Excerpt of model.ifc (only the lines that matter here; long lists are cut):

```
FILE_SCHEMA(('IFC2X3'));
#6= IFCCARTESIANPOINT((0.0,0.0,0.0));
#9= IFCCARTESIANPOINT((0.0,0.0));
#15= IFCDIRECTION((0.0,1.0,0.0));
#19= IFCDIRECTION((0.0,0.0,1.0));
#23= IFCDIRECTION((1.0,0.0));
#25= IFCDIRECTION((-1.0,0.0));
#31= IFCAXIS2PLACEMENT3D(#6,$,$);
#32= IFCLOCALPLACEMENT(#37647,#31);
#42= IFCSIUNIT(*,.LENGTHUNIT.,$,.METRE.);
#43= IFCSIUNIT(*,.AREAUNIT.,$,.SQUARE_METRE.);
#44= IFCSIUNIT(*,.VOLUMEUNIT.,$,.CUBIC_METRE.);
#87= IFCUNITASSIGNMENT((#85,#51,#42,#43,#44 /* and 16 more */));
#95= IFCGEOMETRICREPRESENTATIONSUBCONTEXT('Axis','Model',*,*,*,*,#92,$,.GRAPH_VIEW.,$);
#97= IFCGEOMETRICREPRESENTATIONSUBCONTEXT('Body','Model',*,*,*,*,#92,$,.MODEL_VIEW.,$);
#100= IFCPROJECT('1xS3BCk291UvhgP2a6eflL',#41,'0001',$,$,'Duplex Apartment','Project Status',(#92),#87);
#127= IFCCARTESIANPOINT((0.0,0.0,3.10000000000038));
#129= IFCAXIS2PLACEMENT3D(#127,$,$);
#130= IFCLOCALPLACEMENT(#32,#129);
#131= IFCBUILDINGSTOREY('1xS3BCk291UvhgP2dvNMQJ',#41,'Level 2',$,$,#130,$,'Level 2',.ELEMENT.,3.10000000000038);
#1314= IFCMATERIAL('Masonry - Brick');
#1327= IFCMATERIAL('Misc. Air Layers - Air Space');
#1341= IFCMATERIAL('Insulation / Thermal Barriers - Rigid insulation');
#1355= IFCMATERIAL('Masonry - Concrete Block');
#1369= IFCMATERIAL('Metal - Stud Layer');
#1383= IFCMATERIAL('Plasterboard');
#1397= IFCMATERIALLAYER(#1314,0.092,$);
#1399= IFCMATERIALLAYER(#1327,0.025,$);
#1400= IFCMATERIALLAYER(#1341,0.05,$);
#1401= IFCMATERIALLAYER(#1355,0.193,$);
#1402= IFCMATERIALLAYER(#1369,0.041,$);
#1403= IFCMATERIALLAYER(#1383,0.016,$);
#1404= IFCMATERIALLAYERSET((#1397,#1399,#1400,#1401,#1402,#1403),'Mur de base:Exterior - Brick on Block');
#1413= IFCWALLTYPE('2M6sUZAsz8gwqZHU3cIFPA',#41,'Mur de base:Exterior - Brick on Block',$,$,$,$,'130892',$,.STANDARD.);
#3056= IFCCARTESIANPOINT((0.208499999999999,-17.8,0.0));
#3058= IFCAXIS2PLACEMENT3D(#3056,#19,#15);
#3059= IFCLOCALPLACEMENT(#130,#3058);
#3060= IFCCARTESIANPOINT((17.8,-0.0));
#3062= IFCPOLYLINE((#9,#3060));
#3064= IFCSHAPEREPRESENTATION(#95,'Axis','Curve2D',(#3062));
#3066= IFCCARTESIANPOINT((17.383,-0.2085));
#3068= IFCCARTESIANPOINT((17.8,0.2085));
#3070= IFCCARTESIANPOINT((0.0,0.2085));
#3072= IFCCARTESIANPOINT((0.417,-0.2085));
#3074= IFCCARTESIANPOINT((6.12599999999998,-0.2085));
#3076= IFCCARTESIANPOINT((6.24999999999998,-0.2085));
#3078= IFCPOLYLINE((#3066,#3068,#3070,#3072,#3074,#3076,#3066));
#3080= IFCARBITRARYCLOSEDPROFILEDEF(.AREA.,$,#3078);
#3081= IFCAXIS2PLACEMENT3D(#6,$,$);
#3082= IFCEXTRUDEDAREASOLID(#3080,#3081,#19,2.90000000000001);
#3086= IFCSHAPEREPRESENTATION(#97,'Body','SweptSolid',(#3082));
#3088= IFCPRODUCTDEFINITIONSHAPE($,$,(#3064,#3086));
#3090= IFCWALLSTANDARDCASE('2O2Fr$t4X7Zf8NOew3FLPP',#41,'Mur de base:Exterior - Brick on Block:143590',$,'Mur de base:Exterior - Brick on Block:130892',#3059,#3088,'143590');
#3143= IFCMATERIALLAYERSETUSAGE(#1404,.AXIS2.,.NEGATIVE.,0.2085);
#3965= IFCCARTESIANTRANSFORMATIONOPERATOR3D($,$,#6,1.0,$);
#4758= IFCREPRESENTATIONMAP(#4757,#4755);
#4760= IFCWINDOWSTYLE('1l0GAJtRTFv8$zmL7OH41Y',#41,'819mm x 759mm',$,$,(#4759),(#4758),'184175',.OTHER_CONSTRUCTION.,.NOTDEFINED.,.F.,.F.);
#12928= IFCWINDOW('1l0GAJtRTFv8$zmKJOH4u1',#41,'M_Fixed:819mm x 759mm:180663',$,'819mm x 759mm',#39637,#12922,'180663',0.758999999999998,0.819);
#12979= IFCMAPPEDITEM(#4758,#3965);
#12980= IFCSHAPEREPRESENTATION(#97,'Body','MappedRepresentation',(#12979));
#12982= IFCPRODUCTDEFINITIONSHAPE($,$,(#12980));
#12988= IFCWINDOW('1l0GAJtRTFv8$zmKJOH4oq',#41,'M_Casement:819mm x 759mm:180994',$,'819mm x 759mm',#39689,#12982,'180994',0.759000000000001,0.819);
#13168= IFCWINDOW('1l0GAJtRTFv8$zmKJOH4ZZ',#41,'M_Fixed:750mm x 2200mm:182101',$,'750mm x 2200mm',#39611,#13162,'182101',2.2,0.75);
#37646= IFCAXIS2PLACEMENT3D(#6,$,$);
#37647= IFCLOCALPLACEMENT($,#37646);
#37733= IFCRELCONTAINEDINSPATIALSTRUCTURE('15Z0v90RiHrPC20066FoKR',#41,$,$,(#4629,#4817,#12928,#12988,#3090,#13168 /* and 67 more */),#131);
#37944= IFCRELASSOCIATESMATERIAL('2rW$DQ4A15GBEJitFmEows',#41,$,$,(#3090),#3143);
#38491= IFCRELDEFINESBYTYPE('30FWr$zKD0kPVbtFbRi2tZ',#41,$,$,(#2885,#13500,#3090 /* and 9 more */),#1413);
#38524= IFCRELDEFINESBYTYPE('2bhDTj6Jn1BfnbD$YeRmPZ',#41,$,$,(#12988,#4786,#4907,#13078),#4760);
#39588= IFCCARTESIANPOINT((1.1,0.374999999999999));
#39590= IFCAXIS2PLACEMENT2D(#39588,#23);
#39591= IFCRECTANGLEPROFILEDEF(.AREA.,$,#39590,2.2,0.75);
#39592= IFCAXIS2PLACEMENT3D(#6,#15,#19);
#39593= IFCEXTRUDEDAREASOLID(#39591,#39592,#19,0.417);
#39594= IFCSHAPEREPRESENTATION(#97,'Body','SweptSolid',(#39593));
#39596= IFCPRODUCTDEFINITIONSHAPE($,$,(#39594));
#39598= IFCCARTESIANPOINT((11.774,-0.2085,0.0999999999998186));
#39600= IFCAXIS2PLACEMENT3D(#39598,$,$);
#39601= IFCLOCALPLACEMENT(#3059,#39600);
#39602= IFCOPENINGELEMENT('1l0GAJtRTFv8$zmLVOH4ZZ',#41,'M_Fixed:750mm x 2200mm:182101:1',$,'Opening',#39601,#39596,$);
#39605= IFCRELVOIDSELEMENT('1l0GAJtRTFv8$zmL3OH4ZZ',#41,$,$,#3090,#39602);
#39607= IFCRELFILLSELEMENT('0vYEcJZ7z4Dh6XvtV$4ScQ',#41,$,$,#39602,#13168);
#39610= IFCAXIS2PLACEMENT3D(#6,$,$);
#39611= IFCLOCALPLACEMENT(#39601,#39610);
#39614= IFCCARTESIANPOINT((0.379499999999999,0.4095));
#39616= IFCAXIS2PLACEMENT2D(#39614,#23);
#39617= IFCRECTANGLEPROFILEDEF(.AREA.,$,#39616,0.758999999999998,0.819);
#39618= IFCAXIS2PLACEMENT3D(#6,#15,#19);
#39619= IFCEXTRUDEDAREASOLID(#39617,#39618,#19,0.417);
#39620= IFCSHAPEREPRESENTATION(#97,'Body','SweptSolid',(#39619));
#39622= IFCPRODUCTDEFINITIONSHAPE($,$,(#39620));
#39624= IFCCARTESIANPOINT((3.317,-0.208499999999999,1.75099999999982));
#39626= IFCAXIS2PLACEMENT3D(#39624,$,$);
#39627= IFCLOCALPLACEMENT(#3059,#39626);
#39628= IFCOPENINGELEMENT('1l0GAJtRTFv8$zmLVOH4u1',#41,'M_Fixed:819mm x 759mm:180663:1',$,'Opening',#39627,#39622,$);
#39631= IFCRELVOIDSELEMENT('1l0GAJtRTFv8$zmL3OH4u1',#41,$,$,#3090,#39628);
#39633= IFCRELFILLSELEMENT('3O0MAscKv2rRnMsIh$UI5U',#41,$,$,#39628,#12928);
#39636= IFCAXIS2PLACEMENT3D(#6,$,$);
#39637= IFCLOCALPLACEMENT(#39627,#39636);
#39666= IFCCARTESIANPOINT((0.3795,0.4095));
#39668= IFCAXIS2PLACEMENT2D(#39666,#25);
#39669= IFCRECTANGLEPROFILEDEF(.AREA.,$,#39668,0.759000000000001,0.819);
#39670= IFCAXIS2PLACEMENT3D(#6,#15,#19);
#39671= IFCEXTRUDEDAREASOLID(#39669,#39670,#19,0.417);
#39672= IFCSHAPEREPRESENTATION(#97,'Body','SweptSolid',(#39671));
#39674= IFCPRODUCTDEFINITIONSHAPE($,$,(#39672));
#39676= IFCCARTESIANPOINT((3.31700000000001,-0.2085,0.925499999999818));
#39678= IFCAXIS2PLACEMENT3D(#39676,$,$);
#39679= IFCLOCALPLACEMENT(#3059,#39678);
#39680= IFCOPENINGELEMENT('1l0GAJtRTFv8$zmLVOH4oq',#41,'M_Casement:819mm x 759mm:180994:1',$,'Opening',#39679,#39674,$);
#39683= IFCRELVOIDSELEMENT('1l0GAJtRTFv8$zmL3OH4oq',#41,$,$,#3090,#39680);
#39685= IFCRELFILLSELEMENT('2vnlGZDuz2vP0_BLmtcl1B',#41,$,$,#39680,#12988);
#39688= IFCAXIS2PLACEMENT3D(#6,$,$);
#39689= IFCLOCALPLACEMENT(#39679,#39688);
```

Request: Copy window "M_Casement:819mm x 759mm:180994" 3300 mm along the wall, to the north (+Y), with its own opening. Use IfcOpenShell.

```python
import ifcopenshell
import ifcopenshell.api.feature
import ifcopenshell.api.geometry
import ifcopenshell.api.root
import ifcopenshell.geom
import ifcopenshell.util.element
import ifcopenshell.util.placement
import ifcopenshell.util.shape
import ifcopenshell.util.unit

model = ifcopenshell.open("model.ifc")
unit_scale = ifcopenshell.util.unit.calculate_unit_scale(model)
settings = ifcopenshell.geom.settings()


def volume(element):
    """Net volume in cubic metres, openings subtracted."""
    shape = ifcopenshell.geom.create_shape(settings, element)
    return ifcopenshell.util.shape.get_volume(shape.geometry)


def reuse_history(source, copy):
    """copy_class also copies each property set's owner history, people and application; keep the originals."""
    for rel in copy.IsDefinedBy:
        if rel.is_a("IfcRelDefinesByProperties") and (history := rel.RelatingPropertyDefinition.OwnerHistory):
            rel.RelatingPropertyDefinition.OwnerHistory = source.OwnerHistory
            ifcopenshell.util.element.remove_deep2(model, history)


window = model.by_guid("1l0GAJtRTFv8$zmKJOH4oq")
opening = window.FillsVoids[0].RelatingOpeningElement
wall = opening.VoidsElements[0].RelatingBuildingElement
before = volume(wall)
shift = ifcopenshell.util.placement.get_local_placement(wall.ObjectPlacement)[:3, 0] * 3.3 / unit_scale

# copy_class copies the void relationship, type, container and properties, but no geometry.
new_opening = ifcopenshell.api.root.copy_class(model, product=opening)
new_opening.Representation = ifcopenshell.util.element.copy_deep(
    model, opening.Representation, exclude=["IfcGeometricRepresentationContext", "IfcRepresentationMap"]
)
new_opening.Name = "M_Casement:819mm x 759mm"
new_window = ifcopenshell.api.root.copy_class(model, product=window)
new_window.Representation = ifcopenshell.util.element.copy_deep(
    model, window.Representation, exclude=["IfcGeometricRepresentationContext", "IfcRepresentationMap"]
)
new_window.Name = "M_Casement:819mm x 759mm"
new_window.Tag = None
reuse_history(window, new_window)
fills = ifcopenshell.api.feature.add_filling(model, opening=new_opening, element=new_window)
fills.OwnerHistory = new_window.OwnerHistory  # required in IFC2X3

for old, new in ((opening, new_opening), (window, new_window)):
    matrix = ifcopenshell.util.placement.get_local_placement(old.ObjectPlacement)
    matrix[:3, 3] += shift
    ifcopenshell.api.geometry.edit_object_placement(model, product=new, matrix=matrix, is_si=False)

after = volume(wall)

print(f"wall volume {before:.3f} -> {after:.3f} m3")

model.write("model-out.ifc")
```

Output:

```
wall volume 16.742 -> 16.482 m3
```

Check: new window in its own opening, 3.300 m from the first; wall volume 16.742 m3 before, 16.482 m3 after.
